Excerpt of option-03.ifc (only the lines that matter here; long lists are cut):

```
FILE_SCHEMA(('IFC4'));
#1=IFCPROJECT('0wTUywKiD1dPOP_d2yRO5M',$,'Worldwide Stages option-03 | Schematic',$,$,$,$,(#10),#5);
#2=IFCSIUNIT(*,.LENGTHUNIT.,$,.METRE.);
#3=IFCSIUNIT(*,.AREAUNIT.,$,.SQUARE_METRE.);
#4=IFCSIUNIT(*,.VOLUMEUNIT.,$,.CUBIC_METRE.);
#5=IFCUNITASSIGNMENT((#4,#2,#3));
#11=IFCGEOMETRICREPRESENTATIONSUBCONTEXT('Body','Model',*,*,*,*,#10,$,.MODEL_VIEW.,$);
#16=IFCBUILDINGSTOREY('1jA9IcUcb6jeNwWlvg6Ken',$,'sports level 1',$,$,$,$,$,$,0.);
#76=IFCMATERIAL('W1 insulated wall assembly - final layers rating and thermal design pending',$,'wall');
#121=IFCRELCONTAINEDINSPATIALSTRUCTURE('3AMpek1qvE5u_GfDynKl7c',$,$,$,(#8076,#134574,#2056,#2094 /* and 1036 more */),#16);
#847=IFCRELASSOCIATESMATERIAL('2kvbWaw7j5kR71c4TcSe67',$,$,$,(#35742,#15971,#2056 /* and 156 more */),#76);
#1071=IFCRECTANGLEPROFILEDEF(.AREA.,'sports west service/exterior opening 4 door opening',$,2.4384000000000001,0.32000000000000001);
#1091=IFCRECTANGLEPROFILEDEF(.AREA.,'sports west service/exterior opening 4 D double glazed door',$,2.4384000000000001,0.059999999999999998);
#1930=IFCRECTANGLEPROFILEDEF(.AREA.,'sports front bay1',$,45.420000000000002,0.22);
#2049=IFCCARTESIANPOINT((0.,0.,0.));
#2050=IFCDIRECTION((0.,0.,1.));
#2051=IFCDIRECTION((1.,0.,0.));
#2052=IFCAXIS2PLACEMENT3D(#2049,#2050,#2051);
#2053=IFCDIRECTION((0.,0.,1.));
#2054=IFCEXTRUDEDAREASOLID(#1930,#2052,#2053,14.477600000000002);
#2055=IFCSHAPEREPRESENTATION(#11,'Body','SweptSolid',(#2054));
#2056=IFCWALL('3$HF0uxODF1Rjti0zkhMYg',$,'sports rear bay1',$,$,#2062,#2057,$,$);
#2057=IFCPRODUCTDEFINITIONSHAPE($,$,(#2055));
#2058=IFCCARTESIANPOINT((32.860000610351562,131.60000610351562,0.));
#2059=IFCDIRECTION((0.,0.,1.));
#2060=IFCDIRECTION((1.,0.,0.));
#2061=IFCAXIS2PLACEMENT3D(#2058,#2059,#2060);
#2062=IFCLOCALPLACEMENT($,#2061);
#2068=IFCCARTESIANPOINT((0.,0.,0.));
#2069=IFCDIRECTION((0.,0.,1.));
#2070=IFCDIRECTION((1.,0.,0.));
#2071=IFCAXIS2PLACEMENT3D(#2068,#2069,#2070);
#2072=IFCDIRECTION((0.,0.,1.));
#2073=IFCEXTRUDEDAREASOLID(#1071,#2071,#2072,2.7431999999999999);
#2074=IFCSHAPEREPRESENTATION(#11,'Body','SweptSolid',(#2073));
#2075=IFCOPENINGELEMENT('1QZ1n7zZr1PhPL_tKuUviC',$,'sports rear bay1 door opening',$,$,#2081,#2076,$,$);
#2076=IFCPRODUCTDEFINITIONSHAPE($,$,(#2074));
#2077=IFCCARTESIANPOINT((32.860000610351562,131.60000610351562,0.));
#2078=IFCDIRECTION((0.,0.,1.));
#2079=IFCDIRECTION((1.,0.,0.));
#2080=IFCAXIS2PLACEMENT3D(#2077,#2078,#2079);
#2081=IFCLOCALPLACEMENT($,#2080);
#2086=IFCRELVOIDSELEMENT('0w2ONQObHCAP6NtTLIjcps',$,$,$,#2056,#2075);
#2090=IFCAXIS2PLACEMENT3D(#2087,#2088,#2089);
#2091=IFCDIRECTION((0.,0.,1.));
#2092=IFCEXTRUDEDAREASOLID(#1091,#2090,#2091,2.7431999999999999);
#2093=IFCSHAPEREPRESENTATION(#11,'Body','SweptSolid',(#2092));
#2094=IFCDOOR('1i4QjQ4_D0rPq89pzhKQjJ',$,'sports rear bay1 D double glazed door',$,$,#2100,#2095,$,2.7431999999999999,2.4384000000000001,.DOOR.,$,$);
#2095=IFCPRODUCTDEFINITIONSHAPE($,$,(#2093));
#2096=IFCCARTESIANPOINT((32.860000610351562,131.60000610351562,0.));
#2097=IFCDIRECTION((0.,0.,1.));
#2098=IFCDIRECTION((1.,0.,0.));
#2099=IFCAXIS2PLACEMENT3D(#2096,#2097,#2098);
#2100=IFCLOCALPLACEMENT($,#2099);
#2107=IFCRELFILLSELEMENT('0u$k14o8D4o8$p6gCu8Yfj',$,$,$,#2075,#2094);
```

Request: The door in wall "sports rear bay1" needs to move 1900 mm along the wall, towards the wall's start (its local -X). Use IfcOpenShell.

```python
import ifcopenshell
import ifcopenshell.api.geometry
import ifcopenshell.util.placement

model = ifcopenshell.open("option-03.ifc")

door = model.by_id(2094)
opening = door.FillsVoids[0].RelatingOpeningElement
wall = opening.VoidsElements[0].RelatingBuildingElement

wall_matrix = ifcopenshell.util.placement.get_local_placement(wall.ObjectPlacement)
shift = wall_matrix[:3, 0] * -1.9
before = ifcopenshell.util.placement.get_local_placement(door.ObjectPlacement)[:3, 3].copy()

# The door is not placed relative to its opening, so move both.
for product in (opening, door):
    matrix = ifcopenshell.util.placement.get_local_placement(product.ObjectPlacement)
    matrix[:3, 3] += shift
    ifcopenshell.api.geometry.edit_object_placement(model, product=product, matrix=matrix, is_si=False)

after = ifcopenshell.util.placement.get_local_placement(door.ObjectPlacement)[:3, 3]
print("door moved by", (after - before).round(3) + 0.0)

model.write("option-03_updated.ifc")
```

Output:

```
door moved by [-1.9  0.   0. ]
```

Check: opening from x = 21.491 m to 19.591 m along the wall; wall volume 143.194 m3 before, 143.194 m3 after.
